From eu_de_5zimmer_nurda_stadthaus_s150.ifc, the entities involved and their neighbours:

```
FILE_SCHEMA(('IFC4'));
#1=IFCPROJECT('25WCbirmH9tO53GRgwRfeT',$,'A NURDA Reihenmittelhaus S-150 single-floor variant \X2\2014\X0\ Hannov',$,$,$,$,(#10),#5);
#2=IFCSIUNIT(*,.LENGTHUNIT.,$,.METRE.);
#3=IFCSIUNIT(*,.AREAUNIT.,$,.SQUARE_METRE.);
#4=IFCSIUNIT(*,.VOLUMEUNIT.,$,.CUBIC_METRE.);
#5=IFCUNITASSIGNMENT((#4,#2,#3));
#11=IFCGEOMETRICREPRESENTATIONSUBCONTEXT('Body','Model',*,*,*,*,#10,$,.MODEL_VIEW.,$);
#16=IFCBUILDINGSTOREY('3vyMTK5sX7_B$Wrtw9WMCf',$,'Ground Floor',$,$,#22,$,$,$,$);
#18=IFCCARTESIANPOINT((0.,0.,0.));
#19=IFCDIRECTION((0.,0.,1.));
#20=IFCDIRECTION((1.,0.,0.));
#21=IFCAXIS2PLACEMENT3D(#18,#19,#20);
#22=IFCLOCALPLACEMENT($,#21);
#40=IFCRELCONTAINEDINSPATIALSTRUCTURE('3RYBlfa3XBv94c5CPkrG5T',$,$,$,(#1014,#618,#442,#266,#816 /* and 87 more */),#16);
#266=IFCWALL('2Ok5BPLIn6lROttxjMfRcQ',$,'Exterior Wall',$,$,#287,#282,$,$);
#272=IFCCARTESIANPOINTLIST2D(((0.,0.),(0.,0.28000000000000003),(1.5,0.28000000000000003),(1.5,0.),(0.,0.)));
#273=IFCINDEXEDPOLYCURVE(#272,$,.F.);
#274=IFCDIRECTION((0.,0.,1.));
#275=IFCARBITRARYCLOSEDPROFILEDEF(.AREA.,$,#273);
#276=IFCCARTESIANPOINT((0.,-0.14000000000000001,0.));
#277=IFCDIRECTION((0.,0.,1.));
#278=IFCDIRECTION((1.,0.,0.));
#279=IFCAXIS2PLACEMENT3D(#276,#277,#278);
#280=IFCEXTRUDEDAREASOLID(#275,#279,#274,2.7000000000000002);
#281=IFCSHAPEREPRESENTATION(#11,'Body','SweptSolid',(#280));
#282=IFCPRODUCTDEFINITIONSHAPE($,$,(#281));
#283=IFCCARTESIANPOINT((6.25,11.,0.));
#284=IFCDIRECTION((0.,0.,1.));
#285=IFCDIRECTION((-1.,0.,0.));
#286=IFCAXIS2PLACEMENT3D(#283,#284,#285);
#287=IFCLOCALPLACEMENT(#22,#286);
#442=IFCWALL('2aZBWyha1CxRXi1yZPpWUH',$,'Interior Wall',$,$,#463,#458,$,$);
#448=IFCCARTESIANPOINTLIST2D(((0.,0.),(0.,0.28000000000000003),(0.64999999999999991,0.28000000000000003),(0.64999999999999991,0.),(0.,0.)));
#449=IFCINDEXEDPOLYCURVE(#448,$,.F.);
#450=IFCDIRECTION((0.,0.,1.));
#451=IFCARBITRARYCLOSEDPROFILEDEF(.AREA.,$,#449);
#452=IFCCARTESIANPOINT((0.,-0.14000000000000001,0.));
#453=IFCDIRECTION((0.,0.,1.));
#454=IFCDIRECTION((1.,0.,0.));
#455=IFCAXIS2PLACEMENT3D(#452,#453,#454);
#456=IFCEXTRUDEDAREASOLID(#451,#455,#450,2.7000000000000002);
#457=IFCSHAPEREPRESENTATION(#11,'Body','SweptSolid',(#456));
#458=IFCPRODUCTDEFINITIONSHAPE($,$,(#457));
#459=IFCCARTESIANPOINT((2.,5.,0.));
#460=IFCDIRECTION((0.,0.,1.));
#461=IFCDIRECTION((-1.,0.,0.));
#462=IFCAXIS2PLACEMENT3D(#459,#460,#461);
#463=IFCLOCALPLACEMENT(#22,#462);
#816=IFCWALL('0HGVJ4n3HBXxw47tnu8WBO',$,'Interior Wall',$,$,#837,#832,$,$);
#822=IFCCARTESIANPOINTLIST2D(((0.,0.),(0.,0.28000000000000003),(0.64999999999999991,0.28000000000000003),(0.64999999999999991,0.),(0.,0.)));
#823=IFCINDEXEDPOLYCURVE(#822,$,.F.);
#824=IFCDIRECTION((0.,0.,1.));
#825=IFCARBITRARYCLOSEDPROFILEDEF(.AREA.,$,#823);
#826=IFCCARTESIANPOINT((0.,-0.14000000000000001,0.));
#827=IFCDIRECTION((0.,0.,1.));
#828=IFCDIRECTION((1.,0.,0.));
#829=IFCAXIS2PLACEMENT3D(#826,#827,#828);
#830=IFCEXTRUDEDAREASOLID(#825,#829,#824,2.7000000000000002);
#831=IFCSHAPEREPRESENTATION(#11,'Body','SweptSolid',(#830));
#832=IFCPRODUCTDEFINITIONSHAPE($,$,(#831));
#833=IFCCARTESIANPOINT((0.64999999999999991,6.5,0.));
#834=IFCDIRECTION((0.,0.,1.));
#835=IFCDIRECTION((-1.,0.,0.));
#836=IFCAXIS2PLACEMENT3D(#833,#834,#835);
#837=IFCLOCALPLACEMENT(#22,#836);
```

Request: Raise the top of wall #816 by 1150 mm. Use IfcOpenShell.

```python
import ifcopenshell
import ifcopenshell.geom
import ifcopenshell.util.representation
import ifcopenshell.util.shape
import ifcopenshell.util.unit

model = ifcopenshell.open("eu_de_5zimmer_nurda_stadthaus_s150.ifc")
unit_scale = ifcopenshell.util.unit.calculate_unit_scale(model)
settings = ifcopenshell.geom.settings()


def volume(element):
    """Net volume in cubic metres, openings subtracted."""
    shape = ifcopenshell.geom.create_shape(settings, element)
    return ifcopenshell.util.shape.get_volume(shape.geometry)


wall = model.by_id(816)
before = volume(wall)

body = ifcopenshell.util.representation.get_representation(wall, "Model", "Body")
solid = body.Items[0]
old_height = solid.Depth
solid.Depth += 1.15 / unit_scale
after = volume(wall)

print(f"height {old_height:g} -> {solid.Depth:g}, volume {before:.3f} -> {after:.3f} m3")

model.write("eu_de_5zimmer_nurda_stadthaus_s150_updated.ifc")
```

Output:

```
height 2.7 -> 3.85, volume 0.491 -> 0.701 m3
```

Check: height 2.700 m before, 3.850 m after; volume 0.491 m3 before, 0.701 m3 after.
